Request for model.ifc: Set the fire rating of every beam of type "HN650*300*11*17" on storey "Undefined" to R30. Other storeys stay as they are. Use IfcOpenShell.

First a look at what the model holds.

```python
import ifcopenshell
import ifcopenshell.util.element

model = ifcopenshell.open("model.ifc")
print(model.schema)
storey = next(s for s in model.by_type("IfcBuildingStorey") if s.Name == "Undefined")
beams = [e for e in ifcopenshell.util.element.get_decomposition(storey) if e.is_a("IfcBeam")]
seen = {}
for e in beams:
    element_type = ifcopenshell.util.element.get_type(e)
    key = (element_type.Name if element_type != e and element_type else None, ifcopenshell.util.element.get_pset(e, "Pset_BeamCommon", "FireRating"))
    seen[key] = seen.get(key, 0) + 1
for (name, value), count in sorted(seen.items(), key=str):
    print(count, "x", name, "|", value)
```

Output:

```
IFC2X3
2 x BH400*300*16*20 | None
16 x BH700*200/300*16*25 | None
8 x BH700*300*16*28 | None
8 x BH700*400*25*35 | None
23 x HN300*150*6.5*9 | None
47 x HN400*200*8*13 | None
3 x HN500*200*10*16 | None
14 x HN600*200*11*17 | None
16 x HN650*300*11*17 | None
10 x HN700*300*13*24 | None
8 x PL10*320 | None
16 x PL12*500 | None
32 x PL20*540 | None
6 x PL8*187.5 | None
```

```python
import ifcopenshell
import ifcopenshell.api.pset
import ifcopenshell.util.element

model = ifcopenshell.open("model.ifc")

storey = next(s for s in model.by_type("IfcBuildingStorey") if s.Name == "Undefined")
beams = [e for e in ifcopenshell.util.element.get_decomposition(storey) if e.is_a("IfcBeam")]

count = 0
for e in beams:
    element_type = ifcopenshell.util.element.get_type(e)
    if element_type in (None, e) or element_type.Name != "HN650*300*11*17":
        continue
    # add_pset returns the element's existing set when there is one.
    pset = ifcopenshell.api.pset.add_pset(model, product=e, name="Pset_BeamCommon")
    ifcopenshell.api.pset.edit_pset(model, pset=pset, properties={"FireRating": "R30"})
    count += 1

print(count, "beams updated")

model.write("model_updated.ifc")
```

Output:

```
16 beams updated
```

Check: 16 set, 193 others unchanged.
